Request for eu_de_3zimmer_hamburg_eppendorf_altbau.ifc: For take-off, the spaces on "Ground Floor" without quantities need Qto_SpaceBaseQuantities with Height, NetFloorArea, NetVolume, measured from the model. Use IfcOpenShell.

First a look at what the model holds.

```python
import ifcopenshell
import ifcopenshell.util.element
import ifcopenshell.util.unit

model = ifcopenshell.open("eu_de_3zimmer_hamburg_eppendorf_altbau.ifc")
print(model.schema)
for unit_type in ("LENGTHUNIT", "AREAUNIT", "VOLUMEUNIT"):
    print(unit_type, ifcopenshell.util.unit.calculate_unit_scale(model, unit_type))
storey = next(s for s in model.by_type("IfcBuildingStorey") if s.Name == "Ground Floor")
spaces = [e for e in ifcopenshell.util.element.get_decomposition(storey) if e.is_a("IfcSpace")]
for e in sorted(spaces, key=lambda e: e.id()):
    print(e.id(), e.is_a(), e.Name, list(ifcopenshell.util.element.get_psets(e, qtos_only=True)), sep=" | ")
```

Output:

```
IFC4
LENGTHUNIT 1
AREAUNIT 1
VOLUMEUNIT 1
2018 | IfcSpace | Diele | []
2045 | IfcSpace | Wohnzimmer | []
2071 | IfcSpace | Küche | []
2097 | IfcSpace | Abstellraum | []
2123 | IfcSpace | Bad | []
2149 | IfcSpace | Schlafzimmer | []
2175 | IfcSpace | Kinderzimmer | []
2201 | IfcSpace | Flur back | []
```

```python
import ifcopenshell
import ifcopenshell.api.pset
import ifcopenshell.geom
import ifcopenshell.util.element
import ifcopenshell.util.shape
import ifcopenshell.util.unit

model = ifcopenshell.open("eu_de_3zimmer_hamburg_eppendorf_altbau.ifc")
unit_scale = ifcopenshell.util.unit.calculate_unit_scale(model)
area_scale = ifcopenshell.util.unit.calculate_unit_scale(model, "AREAUNIT")
volume_scale = ifcopenshell.util.unit.calculate_unit_scale(model, "VOLUMEUNIT")
settings = ifcopenshell.geom.settings()

storey = next(s for s in model.by_type("IfcBuildingStorey") if s.Name == "Ground Floor")
spaces = [e for e in ifcopenshell.util.element.get_decomposition(storey) if e.is_a("IfcSpace")]

for e in sorted(spaces, key=lambda e: e.id()):
    if ifcopenshell.util.element.get_psets(e, qtos_only=True, should_inherit=False):
        continue
    # Geometry comes back in metres, in the element's own axes.
    shape = ifcopenshell.geom.create_shape(settings, e)
    values = {
        "Height": ifcopenshell.util.shape.get_z(shape.geometry) / unit_scale,
        "NetFloorArea": ifcopenshell.util.shape.get_footprint_area(shape.geometry) / area_scale,
        "NetVolume": ifcopenshell.util.shape.get_volume(shape.geometry) / volume_scale,
    }
    qto = ifcopenshell.api.pset.add_qto(model, product=e, name="Qto_SpaceBaseQuantities")
    ifcopenshell.api.pset.edit_qto(model, qto=qto, properties=values)
    print(e.id(), {k: round(v, 3) for k, v in values.items()})

model.write("eu_de_3zimmer_hamburg_eppendorf_altbau_edited.ifc")
```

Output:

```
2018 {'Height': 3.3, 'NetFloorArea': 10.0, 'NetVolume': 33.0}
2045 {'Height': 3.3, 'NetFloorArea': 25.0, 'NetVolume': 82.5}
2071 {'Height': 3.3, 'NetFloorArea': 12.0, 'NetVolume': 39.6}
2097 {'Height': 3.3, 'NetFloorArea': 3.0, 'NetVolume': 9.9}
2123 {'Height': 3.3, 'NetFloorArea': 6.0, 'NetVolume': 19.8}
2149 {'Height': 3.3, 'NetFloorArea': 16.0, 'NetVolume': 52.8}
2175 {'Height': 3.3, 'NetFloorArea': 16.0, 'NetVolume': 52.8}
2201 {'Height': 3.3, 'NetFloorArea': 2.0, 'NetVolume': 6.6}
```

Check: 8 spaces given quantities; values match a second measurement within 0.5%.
